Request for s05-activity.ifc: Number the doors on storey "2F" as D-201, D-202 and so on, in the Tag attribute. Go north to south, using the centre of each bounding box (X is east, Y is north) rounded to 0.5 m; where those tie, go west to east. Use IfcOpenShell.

First a look at what the model holds.

```python
import ifcopenshell
import ifcopenshell.util.element
import ifcopenshell.util.placement

model = ifcopenshell.open("s05-activity.ifc")
print(model.schema)
storey = next(s for s in model.by_type("IfcBuildingStorey") if s.Name == "2F")
doors = [e for e in ifcopenshell.util.element.get_decomposition(storey) if e.is_a("IfcDoor")]
for e in sorted(doors, key=lambda e: e.id()):
    origin = ifcopenshell.util.placement.get_local_placement(e.ObjectPlacement)[:3, 3]
    print(e.id(), e.Tag, e.Name, origin.round(2) + 0.0, sep=" | ")
```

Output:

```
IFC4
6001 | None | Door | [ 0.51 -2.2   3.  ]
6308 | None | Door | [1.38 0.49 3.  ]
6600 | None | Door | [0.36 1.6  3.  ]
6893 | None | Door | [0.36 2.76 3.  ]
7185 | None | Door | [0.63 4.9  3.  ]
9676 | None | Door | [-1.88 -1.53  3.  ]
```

```python
import ifcopenshell
import ifcopenshell.geom
import ifcopenshell.util.element
import ifcopenshell.util.shape

model = ifcopenshell.open("s05-activity.ifc")
settings = ifcopenshell.geom.settings()
settings.set("use-world-coords", True)


def centre(element):
    shape = ifcopenshell.geom.create_shape(settings, element)
    return ifcopenshell.util.shape.get_bbox_centroid(shape.geometry)


storey = next(s for s in model.by_type("IfcBuildingStorey") if s.Name == "2F")
doors = [e for e in ifcopenshell.util.element.get_decomposition(storey) if e.is_a("IfcDoor")]

# Insertion points can sit at a corner or the storey origin, so sort by the geometry (in metres).
centres = {e: centre(e) for e in doors}
doors.sort(key=lambda e: (-round(centres[e][1] / 0.5), centres[e][0]))

for i, e in enumerate(doors, start=1):
    number = f"D-2{i:02d}"
    e.Tag = number
    print(e.id(), number)

model.write("s05-activity_updated.ifc")
```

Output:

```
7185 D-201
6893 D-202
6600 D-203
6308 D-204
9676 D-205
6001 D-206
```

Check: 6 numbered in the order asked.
